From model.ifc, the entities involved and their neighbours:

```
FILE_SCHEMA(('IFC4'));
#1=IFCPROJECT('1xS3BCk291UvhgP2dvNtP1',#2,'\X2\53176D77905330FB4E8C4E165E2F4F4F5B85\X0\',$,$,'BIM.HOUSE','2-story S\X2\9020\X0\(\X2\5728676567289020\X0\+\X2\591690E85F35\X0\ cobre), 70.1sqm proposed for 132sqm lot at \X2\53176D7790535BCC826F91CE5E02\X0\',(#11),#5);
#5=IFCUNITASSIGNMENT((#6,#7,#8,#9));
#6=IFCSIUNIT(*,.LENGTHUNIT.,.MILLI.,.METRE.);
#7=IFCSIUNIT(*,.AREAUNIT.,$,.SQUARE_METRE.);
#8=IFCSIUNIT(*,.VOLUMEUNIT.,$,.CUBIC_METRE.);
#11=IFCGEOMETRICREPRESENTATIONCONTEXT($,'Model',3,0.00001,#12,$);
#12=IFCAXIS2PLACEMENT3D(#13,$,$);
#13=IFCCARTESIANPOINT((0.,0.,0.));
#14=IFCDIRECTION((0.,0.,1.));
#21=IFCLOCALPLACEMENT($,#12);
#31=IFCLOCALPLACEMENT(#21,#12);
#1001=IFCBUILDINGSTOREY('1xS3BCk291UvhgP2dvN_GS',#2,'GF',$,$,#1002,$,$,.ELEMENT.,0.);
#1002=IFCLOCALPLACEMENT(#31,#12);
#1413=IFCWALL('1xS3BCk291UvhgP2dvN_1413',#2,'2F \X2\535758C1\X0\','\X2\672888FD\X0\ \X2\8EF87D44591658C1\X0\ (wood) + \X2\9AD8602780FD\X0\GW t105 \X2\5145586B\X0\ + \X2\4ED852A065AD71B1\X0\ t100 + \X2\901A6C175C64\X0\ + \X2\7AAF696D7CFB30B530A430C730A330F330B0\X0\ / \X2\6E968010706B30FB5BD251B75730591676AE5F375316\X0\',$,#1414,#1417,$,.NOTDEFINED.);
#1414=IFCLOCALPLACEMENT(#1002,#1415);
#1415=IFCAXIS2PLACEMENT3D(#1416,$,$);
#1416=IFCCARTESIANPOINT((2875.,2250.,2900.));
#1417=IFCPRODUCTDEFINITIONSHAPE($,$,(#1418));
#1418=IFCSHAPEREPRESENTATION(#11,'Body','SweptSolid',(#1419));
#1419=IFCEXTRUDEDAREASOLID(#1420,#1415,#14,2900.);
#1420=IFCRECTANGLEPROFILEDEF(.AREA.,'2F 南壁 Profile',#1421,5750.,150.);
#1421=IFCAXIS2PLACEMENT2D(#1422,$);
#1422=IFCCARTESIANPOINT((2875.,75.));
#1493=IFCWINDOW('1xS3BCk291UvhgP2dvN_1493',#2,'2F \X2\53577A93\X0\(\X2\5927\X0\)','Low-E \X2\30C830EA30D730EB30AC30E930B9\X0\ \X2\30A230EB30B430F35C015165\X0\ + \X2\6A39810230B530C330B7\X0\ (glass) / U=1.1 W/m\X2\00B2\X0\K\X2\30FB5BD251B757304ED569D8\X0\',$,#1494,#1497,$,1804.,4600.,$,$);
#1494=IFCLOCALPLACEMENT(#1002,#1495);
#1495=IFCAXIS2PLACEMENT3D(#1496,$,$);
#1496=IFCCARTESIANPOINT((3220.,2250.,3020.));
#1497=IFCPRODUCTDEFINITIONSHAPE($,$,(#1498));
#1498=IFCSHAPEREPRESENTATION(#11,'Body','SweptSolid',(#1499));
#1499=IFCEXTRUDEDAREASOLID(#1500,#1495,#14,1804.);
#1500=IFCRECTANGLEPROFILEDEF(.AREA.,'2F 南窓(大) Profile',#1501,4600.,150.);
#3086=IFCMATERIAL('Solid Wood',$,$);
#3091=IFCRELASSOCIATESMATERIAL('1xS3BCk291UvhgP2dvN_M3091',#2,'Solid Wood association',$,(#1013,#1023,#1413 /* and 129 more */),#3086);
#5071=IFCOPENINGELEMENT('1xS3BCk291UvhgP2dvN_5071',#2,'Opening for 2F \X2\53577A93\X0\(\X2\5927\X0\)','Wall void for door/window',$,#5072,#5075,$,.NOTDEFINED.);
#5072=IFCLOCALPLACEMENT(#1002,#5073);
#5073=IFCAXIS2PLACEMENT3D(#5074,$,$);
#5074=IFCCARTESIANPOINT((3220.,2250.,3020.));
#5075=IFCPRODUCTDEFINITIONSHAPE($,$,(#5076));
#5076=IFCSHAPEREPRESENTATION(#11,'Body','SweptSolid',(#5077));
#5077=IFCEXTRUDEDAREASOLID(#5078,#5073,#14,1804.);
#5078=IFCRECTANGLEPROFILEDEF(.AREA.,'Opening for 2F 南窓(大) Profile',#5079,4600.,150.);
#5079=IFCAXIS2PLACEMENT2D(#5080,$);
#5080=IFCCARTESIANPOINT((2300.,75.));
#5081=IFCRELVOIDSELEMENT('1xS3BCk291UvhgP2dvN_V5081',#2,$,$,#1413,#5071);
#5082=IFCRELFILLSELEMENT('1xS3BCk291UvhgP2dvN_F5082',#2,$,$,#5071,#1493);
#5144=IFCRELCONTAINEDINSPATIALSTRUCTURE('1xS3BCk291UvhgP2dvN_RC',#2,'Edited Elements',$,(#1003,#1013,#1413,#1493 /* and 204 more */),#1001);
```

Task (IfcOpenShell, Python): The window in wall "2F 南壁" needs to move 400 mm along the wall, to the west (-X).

```python
import ifcopenshell
import ifcopenshell.api.geometry
import ifcopenshell.util.placement
import ifcopenshell.util.unit

model = ifcopenshell.open("model.ifc")
unit_scale = ifcopenshell.util.unit.calculate_unit_scale(model)

window = model.by_guid("1xS3BCk291UvhgP2dvN_1493")
opening = window.FillsVoids[0].RelatingOpeningElement
wall = opening.VoidsElements[0].RelatingBuildingElement

wall_matrix = ifcopenshell.util.placement.get_local_placement(wall.ObjectPlacement)
shift = wall_matrix[:3, 0] * -0.4 / unit_scale
before = ifcopenshell.util.placement.get_local_placement(window.ObjectPlacement)[:3, 3].copy()

# The window is not placed relative to its opening, so move both.
for product in (opening, window):
    matrix = ifcopenshell.util.placement.get_local_placement(product.ObjectPlacement)
    matrix[:3, 3] += shift
    ifcopenshell.api.geometry.edit_object_placement(model, product=product, matrix=matrix, is_si=False)

after = ifcopenshell.util.placement.get_local_placement(window.ObjectPlacement)[:3, 3]
print("window moved by", (after - before).round(3) + 0.0)

model.write("model_rev.ifc")
```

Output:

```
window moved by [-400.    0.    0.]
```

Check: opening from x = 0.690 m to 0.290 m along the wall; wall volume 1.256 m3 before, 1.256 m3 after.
